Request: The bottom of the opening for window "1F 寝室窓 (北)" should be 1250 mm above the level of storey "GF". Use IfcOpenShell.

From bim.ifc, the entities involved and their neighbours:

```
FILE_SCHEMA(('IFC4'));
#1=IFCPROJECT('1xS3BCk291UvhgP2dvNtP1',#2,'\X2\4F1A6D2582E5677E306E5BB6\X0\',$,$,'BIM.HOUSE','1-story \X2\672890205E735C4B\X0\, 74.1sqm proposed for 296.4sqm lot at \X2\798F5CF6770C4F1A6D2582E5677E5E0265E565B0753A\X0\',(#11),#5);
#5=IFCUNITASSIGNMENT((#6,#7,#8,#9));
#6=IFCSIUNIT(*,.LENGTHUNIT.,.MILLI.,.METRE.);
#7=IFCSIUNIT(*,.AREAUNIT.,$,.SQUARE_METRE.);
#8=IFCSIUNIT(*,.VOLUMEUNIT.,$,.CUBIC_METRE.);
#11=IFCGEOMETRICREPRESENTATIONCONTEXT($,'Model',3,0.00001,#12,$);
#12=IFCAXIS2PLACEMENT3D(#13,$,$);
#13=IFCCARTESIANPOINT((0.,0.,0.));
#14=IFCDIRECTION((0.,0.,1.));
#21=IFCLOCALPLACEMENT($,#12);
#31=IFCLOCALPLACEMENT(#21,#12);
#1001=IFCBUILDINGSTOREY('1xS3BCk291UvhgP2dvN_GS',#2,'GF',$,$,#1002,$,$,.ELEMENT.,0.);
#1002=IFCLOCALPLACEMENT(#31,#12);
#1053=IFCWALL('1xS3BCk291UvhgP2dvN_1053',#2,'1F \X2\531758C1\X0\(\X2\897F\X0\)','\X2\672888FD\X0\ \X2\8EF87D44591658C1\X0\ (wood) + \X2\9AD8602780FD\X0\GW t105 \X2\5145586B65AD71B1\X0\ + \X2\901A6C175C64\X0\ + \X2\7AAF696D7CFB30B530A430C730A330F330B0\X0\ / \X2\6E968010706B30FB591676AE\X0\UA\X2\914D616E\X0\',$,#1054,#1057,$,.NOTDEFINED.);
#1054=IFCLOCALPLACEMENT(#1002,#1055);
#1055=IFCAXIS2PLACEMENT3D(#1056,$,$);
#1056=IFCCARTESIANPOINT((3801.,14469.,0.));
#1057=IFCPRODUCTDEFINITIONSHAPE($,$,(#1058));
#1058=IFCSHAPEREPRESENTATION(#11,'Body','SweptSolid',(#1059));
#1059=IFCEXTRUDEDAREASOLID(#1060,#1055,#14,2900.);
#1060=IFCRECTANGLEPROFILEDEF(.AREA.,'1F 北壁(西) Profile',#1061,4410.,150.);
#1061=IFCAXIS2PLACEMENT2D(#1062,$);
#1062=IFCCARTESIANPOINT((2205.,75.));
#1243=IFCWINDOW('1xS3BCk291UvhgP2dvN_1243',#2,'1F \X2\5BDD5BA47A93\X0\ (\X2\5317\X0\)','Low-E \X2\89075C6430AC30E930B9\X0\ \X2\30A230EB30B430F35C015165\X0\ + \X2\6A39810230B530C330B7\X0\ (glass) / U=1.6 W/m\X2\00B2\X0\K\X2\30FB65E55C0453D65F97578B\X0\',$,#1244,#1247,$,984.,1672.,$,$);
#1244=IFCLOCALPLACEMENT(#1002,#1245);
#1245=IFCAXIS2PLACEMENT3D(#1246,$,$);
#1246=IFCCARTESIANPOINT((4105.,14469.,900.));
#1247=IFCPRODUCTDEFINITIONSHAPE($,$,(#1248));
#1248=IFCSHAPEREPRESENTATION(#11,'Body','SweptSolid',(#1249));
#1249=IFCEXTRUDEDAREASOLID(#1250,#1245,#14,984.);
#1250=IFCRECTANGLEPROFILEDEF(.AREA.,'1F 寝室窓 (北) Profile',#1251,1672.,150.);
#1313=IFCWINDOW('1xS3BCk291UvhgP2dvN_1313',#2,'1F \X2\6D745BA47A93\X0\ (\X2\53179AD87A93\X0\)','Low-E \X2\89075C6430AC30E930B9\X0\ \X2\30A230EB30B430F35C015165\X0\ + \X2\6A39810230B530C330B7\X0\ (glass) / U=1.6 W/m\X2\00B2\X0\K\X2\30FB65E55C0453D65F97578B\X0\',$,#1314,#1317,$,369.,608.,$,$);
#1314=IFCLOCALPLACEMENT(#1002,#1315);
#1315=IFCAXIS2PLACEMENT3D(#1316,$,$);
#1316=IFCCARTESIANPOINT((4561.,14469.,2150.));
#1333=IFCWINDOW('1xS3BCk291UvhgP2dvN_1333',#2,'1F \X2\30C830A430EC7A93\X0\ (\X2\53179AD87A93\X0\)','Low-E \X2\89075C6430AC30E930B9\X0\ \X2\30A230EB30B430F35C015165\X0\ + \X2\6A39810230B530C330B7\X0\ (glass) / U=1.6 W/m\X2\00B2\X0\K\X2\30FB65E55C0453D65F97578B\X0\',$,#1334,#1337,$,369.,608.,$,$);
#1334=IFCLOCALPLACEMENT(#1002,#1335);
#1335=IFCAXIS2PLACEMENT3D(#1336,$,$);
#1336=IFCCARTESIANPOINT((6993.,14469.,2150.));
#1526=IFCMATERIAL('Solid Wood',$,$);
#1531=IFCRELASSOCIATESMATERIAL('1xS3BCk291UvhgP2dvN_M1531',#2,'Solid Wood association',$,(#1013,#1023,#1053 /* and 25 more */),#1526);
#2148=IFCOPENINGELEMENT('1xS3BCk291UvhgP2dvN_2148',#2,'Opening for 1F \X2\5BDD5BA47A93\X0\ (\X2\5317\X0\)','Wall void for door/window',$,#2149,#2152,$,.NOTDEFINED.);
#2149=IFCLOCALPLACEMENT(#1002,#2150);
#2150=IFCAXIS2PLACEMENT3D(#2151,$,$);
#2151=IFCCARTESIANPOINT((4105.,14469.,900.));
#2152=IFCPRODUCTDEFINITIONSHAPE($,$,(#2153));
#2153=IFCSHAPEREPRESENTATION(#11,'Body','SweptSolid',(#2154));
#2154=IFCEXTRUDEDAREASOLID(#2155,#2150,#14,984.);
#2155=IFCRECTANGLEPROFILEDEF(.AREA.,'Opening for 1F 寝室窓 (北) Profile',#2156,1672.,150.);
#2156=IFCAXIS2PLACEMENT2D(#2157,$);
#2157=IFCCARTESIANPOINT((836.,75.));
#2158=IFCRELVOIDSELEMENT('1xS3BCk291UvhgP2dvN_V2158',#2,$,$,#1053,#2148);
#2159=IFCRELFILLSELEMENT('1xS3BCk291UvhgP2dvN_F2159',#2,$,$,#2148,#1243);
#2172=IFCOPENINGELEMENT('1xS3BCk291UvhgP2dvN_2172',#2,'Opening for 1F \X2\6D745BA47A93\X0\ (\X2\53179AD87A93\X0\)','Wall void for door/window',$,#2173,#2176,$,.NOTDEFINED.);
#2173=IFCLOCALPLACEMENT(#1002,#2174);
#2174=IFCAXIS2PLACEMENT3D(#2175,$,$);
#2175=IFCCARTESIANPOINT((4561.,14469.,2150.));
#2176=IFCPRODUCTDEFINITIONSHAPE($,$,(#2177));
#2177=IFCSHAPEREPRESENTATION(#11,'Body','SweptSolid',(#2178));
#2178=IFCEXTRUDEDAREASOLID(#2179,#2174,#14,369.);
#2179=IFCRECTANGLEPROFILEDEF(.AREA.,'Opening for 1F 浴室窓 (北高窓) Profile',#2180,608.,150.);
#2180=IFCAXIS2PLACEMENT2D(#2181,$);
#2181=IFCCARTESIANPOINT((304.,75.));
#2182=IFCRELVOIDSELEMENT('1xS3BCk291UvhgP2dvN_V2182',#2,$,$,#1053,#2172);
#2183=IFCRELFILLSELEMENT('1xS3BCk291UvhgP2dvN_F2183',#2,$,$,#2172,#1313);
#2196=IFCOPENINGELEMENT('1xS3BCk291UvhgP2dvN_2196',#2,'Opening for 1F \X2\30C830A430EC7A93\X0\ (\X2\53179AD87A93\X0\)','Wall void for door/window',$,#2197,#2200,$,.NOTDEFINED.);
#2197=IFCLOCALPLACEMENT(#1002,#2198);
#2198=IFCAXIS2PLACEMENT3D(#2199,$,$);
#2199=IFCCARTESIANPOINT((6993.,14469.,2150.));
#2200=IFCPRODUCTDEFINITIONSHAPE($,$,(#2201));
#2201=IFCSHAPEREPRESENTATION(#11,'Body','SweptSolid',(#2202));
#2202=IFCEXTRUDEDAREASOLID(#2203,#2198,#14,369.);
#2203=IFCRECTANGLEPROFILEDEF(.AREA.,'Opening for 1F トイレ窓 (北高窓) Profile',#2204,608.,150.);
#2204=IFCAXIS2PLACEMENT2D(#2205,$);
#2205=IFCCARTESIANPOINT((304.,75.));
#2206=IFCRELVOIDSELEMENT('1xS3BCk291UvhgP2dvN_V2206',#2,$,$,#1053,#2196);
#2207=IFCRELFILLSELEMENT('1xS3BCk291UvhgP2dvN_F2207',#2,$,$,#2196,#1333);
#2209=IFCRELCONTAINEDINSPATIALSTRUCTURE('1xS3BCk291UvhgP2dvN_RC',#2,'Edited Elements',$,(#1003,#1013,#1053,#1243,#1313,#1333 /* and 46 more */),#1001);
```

```python
import numpy as np
import ifcopenshell
import ifcopenshell.api.geometry
import ifcopenshell.geom
import ifcopenshell.util.element
import ifcopenshell.util.placement
import ifcopenshell.util.shape
import ifcopenshell.util.unit

model = ifcopenshell.open("bim.ifc")
unit_scale = ifcopenshell.util.unit.calculate_unit_scale(model)

window = model.by_guid("1xS3BCk291UvhgP2dvN_1243")
opening = window.FillsVoids[0].RelatingOpeningElement
storey = ifcopenshell.util.element.get_container(window, ifc_class="IfcBuildingStorey")
level = ifcopenshell.util.placement.get_local_placement(storey.ObjectPlacement)[2, 3]

# The opening's origin need not be at the sill, so measure its lowest point.
shape = ifcopenshell.geom.create_shape(ifcopenshell.geom.settings(), opening)
bottom = ifcopenshell.util.shape.get_shape_bottom_elevation(shape, shape.geometry) / unit_scale
dz = level + 1250.0 - bottom

shift = np.array([0.0, 0.0, dz])
# The window is not placed relative to its opening, so move both.
for product in (opening, window):
    matrix = ifcopenshell.util.placement.get_local_placement(product.ObjectPlacement)
    matrix[:3, 3] += shift
    ifcopenshell.api.geometry.edit_object_placement(model, product=product, matrix=matrix, is_si=False)

print(f"moved by {dz * unit_scale:+.3f} m")

model.write("bim_rev.ifc")
```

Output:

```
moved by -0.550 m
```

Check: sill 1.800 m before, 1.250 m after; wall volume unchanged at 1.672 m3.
